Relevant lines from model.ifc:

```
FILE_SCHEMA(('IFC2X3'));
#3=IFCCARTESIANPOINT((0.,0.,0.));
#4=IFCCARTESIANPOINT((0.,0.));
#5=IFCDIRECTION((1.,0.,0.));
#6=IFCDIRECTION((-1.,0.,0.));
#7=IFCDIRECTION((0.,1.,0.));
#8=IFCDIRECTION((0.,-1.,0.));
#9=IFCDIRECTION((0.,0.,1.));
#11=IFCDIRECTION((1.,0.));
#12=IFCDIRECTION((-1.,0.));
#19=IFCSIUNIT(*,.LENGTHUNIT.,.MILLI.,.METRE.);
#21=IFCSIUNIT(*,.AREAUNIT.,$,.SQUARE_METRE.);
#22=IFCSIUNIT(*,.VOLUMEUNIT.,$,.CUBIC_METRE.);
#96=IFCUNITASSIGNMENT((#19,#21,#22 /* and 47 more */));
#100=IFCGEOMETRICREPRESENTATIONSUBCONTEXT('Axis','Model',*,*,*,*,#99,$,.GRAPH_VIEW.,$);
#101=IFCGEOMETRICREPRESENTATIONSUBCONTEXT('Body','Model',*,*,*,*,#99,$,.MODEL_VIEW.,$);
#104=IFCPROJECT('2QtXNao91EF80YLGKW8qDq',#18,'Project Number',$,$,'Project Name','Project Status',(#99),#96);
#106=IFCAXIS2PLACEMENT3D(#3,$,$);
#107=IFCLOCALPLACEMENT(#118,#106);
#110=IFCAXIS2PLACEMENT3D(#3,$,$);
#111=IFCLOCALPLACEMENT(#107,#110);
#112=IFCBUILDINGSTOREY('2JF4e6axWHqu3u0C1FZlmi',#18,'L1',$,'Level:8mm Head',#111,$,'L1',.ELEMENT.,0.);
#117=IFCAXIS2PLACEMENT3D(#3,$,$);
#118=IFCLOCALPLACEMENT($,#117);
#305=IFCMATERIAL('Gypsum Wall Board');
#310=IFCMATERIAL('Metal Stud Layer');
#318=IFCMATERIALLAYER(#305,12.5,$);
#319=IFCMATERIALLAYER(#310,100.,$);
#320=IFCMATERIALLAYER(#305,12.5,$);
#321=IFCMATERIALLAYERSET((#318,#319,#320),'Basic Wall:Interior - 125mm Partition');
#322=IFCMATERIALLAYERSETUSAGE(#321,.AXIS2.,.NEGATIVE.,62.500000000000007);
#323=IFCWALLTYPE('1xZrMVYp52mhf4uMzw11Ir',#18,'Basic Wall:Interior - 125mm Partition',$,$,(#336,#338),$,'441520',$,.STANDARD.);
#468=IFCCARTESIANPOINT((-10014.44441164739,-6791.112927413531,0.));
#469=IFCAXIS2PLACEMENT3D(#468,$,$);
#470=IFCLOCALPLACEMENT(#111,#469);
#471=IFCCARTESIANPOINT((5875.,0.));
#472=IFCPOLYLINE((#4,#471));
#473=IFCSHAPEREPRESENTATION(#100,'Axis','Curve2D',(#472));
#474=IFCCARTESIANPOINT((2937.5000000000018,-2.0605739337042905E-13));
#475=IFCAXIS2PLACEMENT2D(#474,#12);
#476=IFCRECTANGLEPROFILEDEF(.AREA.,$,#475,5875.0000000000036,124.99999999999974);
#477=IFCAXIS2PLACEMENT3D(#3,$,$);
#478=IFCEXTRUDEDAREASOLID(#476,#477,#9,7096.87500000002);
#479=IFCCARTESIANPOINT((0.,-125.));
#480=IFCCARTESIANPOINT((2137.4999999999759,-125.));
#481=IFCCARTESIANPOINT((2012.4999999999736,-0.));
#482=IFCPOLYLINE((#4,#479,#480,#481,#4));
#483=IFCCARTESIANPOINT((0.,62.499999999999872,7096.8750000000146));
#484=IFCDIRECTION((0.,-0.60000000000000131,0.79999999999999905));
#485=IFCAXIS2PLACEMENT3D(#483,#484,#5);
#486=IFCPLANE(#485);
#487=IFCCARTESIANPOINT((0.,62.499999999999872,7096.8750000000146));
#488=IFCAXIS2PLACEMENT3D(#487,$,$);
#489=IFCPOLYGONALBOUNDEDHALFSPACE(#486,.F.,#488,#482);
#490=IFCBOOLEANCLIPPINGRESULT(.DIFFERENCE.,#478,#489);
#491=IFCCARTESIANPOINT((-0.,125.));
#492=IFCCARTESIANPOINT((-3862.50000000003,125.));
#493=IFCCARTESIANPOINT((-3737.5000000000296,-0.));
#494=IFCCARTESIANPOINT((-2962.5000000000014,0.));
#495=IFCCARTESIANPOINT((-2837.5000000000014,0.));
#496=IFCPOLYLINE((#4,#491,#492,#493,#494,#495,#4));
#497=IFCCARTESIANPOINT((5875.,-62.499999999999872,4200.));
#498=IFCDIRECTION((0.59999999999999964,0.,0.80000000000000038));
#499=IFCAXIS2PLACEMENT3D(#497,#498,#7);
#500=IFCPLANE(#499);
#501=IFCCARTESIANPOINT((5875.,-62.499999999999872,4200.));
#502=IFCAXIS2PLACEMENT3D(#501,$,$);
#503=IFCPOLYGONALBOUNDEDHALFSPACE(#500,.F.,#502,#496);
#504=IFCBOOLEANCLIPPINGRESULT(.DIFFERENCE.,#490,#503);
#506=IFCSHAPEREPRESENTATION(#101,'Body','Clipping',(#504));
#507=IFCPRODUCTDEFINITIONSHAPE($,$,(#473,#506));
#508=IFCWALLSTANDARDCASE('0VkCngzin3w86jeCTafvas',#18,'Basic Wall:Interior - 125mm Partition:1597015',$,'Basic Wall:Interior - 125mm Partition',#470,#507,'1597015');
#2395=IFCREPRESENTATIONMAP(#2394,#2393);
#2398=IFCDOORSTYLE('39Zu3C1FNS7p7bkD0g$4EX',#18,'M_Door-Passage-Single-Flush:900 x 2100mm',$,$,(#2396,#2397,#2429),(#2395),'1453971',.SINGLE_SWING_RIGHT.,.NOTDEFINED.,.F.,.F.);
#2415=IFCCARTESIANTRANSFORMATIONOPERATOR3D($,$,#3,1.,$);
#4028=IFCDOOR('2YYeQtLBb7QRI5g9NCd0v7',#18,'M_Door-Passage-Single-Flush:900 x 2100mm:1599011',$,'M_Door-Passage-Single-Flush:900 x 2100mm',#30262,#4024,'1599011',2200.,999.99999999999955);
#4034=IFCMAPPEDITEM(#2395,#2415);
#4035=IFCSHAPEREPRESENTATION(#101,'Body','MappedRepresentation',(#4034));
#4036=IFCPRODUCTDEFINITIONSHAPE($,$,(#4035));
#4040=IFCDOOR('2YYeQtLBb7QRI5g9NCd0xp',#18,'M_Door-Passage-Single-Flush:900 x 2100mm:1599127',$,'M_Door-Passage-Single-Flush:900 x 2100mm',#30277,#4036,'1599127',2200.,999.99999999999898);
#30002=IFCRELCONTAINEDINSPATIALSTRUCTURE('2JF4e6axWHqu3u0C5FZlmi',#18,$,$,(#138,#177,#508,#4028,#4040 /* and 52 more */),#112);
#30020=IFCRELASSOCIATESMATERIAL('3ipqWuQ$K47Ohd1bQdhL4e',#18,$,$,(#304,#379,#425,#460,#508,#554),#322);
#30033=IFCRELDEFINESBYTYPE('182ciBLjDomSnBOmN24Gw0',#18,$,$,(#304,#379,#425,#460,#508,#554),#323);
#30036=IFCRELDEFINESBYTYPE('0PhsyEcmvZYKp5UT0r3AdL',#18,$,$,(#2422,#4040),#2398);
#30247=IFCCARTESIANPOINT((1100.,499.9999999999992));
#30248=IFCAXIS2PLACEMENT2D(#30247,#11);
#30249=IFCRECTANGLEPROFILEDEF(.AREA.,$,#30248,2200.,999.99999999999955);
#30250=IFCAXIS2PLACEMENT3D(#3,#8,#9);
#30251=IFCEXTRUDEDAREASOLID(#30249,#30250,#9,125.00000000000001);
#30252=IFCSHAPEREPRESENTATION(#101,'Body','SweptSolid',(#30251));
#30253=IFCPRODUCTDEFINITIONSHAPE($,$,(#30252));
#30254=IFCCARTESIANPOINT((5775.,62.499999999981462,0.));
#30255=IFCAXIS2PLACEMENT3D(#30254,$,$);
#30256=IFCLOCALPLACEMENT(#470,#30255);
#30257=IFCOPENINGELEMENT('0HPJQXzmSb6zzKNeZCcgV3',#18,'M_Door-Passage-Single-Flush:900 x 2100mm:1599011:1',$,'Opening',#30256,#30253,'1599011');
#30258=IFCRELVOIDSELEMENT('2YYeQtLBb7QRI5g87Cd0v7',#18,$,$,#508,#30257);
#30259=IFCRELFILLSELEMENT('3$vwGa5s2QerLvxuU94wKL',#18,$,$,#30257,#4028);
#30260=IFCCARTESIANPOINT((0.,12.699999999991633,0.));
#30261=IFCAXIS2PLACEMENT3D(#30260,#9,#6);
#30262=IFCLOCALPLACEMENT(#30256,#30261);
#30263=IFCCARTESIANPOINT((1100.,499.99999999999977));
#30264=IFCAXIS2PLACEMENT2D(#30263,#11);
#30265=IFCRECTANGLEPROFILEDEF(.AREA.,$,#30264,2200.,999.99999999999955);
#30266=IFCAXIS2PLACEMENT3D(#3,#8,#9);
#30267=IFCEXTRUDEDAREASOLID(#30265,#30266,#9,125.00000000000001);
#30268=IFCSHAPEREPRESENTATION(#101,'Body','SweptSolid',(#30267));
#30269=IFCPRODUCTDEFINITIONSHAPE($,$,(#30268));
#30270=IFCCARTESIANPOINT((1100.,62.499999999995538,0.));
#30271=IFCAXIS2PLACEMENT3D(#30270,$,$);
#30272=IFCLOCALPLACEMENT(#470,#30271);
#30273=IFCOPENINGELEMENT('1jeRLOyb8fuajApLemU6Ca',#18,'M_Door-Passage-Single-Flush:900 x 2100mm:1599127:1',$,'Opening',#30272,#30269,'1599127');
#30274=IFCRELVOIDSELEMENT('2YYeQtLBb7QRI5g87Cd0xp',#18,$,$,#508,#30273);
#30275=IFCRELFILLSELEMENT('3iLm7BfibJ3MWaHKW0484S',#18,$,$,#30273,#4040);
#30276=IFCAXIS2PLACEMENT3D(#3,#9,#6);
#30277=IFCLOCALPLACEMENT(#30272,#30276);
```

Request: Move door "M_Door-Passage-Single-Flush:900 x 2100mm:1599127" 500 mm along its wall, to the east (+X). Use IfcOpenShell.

```python
import ifcopenshell
import ifcopenshell.api.geometry
import ifcopenshell.util.placement
import ifcopenshell.util.unit

model = ifcopenshell.open("model.ifc")
unit_scale = ifcopenshell.util.unit.calculate_unit_scale(model)

door = model.by_guid("2YYeQtLBb7QRI5g9NCd0xp")
opening = door.FillsVoids[0].RelatingOpeningElement
wall = opening.VoidsElements[0].RelatingBuildingElement

wall_matrix = ifcopenshell.util.placement.get_local_placement(wall.ObjectPlacement)
shift = wall_matrix[:3, 0] * 0.5 / unit_scale
before = ifcopenshell.util.placement.get_local_placement(door.ObjectPlacement)[:3, 3].copy()

# The door is placed relative to its opening, so it follows when the opening moves.
matrix = ifcopenshell.util.placement.get_local_placement(opening.ObjectPlacement)
matrix[:3, 3] += shift
ifcopenshell.api.geometry.edit_object_placement(
    model, product=opening, matrix=matrix, is_si=False, should_transform_children=True
)

after = ifcopenshell.util.placement.get_local_placement(door.ObjectPlacement)[:3, 3]
print("door moved by", (after - before).round(3) + 0.0)

model.write("model_v2.ifc")
```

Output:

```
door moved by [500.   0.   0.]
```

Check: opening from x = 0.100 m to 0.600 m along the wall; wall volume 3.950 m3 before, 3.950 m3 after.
